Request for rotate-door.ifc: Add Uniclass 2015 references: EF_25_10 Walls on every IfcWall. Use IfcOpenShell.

First a look at what the model holds.

```python
import ifcopenshell

model = ifcopenshell.open("rotate-door.ifc")
print(model.schema)
print("classifications:", [c.Name for c in model.by_type("IfcClassification")])
for ifc_class in ("IfcDoor", "IfcRoof", "IfcStair", "IfcWall", "IfcWindow"):
    print(ifc_class, len(model.by_type(ifc_class)))
```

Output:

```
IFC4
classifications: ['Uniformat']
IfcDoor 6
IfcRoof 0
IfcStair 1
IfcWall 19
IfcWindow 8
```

```python
import ifcopenshell
import ifcopenshell.api.classification

model = ifcopenshell.open("rotate-door.ifc")

system = ifcopenshell.api.classification.add_classification(model, classification="Uniclass 2015")

codes = {
    "IfcWall": ("EF_25_10", "Walls"),
}
for ifc_class, (code, name) in codes.items():
    products = model.by_type(ifc_class)
    ifcopenshell.api.classification.add_reference(
        model, products=products, classification=system, identification=code, name=name
    )
    print(code, len(products))

model.write("rotate-door-out.ifc")
```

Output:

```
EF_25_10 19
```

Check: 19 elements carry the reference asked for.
